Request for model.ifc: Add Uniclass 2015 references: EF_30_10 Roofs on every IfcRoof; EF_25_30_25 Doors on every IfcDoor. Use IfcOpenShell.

First a look at what the model holds.

```python
import ifcopenshell

model = ifcopenshell.open("model.ifc")
print(model.schema)
print("classifications:", [c.Name for c in model.by_type("IfcClassification")])
for ifc_class in ("IfcDoor", "IfcRoof", "IfcStair", "IfcWall", "IfcWindow"):
    print(ifc_class, len(model.by_type(ifc_class)))
```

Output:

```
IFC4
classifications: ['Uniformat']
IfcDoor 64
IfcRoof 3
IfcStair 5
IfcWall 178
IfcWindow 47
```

```python
import ifcopenshell
import ifcopenshell.api.classification

model = ifcopenshell.open("model.ifc")

system = ifcopenshell.api.classification.add_classification(model, classification="Uniclass 2015")

codes = {
    "IfcRoof": ("EF_30_10", "Roofs"),
    "IfcDoor": ("EF_25_30_25", "Doors"),
}
for ifc_class, (code, name) in codes.items():
    products = model.by_type(ifc_class)
    ifcopenshell.api.classification.add_reference(
        model, products=products, classification=system, identification=code, name=name
    )
    print(code, len(products))

model.write("model-out.ifc")
```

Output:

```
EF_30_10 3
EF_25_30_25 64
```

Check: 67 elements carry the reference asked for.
